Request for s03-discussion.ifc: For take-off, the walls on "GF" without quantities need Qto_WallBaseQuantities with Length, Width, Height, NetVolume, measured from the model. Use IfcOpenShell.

First a look at what the model holds.

```python
import ifcopenshell
import ifcopenshell.util.element
import ifcopenshell.util.unit

model = ifcopenshell.open("s03-discussion.ifc")
print(model.schema)
for unit_type in ("LENGTHUNIT", "AREAUNIT", "VOLUMEUNIT"):
    print(unit_type, ifcopenshell.util.unit.calculate_unit_scale(model, unit_type))
storey = next(s for s in model.by_type("IfcBuildingStorey") if s.Name == "GF")
walls = [e for e in ifcopenshell.util.element.get_decomposition(storey) if e.is_a("IfcWall")]
for e in sorted(walls, key=lambda e: e.id()):
    print(e.id(), e.is_a(), e.Name, list(ifcopenshell.util.element.get_psets(e, qtos_only=True)), sep=" | ")
```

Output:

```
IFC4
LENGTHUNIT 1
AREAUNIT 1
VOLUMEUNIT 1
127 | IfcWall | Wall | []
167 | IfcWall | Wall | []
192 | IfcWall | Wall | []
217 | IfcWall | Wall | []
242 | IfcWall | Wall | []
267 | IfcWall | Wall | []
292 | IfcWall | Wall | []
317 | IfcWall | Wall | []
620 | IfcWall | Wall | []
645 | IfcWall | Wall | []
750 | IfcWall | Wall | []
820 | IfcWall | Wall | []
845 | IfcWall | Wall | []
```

```python
import ifcopenshell
import ifcopenshell.api.pset
import ifcopenshell.geom
import ifcopenshell.util.element
import ifcopenshell.util.shape
import ifcopenshell.util.unit

model = ifcopenshell.open("s03-discussion.ifc")
unit_scale = ifcopenshell.util.unit.calculate_unit_scale(model)
volume_scale = ifcopenshell.util.unit.calculate_unit_scale(model, "VOLUMEUNIT")
settings = ifcopenshell.geom.settings()

storey = next(s for s in model.by_type("IfcBuildingStorey") if s.Name == "GF")
walls = [e for e in ifcopenshell.util.element.get_decomposition(storey) if e.is_a("IfcWall")]

for e in sorted(walls, key=lambda e: e.id()):
    if ifcopenshell.util.element.get_psets(e, qtos_only=True, should_inherit=False):
        continue
    # Geometry comes back in metres, in the element's own axes.
    shape = ifcopenshell.geom.create_shape(settings, e)
    values = {
        "Length": ifcopenshell.util.shape.get_x(shape.geometry) / unit_scale,
        "Width": ifcopenshell.util.shape.get_y(shape.geometry) / unit_scale,
        "Height": ifcopenshell.util.shape.get_z(shape.geometry) / unit_scale,
        "NetVolume": ifcopenshell.util.shape.get_volume(shape.geometry) / volume_scale,
    }
    qto = ifcopenshell.api.pset.add_qto(model, product=e, name="Qto_WallBaseQuantities")
    ifcopenshell.api.pset.edit_qto(model, qto=qto, properties=values)
    print(e.id(), {k: round(v, 3) for k, v in values.items()})

model.write("s03-discussion_rev.ifc")
```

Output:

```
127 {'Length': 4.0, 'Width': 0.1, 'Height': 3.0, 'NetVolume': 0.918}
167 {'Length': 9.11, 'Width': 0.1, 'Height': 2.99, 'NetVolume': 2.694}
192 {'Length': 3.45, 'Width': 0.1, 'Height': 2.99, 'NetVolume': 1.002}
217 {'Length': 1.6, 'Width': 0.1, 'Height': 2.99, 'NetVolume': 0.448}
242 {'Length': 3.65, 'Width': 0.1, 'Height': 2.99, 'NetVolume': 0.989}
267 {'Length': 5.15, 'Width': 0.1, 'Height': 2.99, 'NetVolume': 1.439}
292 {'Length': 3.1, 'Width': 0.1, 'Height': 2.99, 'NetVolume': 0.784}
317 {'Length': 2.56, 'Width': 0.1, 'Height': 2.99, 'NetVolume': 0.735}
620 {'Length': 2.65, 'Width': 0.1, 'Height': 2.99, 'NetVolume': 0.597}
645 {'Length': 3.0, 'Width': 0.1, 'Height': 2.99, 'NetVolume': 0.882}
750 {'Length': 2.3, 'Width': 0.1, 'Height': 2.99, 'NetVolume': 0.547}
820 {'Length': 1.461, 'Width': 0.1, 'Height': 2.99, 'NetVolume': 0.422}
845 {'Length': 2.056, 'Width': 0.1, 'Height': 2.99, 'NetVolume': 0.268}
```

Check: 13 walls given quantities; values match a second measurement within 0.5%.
